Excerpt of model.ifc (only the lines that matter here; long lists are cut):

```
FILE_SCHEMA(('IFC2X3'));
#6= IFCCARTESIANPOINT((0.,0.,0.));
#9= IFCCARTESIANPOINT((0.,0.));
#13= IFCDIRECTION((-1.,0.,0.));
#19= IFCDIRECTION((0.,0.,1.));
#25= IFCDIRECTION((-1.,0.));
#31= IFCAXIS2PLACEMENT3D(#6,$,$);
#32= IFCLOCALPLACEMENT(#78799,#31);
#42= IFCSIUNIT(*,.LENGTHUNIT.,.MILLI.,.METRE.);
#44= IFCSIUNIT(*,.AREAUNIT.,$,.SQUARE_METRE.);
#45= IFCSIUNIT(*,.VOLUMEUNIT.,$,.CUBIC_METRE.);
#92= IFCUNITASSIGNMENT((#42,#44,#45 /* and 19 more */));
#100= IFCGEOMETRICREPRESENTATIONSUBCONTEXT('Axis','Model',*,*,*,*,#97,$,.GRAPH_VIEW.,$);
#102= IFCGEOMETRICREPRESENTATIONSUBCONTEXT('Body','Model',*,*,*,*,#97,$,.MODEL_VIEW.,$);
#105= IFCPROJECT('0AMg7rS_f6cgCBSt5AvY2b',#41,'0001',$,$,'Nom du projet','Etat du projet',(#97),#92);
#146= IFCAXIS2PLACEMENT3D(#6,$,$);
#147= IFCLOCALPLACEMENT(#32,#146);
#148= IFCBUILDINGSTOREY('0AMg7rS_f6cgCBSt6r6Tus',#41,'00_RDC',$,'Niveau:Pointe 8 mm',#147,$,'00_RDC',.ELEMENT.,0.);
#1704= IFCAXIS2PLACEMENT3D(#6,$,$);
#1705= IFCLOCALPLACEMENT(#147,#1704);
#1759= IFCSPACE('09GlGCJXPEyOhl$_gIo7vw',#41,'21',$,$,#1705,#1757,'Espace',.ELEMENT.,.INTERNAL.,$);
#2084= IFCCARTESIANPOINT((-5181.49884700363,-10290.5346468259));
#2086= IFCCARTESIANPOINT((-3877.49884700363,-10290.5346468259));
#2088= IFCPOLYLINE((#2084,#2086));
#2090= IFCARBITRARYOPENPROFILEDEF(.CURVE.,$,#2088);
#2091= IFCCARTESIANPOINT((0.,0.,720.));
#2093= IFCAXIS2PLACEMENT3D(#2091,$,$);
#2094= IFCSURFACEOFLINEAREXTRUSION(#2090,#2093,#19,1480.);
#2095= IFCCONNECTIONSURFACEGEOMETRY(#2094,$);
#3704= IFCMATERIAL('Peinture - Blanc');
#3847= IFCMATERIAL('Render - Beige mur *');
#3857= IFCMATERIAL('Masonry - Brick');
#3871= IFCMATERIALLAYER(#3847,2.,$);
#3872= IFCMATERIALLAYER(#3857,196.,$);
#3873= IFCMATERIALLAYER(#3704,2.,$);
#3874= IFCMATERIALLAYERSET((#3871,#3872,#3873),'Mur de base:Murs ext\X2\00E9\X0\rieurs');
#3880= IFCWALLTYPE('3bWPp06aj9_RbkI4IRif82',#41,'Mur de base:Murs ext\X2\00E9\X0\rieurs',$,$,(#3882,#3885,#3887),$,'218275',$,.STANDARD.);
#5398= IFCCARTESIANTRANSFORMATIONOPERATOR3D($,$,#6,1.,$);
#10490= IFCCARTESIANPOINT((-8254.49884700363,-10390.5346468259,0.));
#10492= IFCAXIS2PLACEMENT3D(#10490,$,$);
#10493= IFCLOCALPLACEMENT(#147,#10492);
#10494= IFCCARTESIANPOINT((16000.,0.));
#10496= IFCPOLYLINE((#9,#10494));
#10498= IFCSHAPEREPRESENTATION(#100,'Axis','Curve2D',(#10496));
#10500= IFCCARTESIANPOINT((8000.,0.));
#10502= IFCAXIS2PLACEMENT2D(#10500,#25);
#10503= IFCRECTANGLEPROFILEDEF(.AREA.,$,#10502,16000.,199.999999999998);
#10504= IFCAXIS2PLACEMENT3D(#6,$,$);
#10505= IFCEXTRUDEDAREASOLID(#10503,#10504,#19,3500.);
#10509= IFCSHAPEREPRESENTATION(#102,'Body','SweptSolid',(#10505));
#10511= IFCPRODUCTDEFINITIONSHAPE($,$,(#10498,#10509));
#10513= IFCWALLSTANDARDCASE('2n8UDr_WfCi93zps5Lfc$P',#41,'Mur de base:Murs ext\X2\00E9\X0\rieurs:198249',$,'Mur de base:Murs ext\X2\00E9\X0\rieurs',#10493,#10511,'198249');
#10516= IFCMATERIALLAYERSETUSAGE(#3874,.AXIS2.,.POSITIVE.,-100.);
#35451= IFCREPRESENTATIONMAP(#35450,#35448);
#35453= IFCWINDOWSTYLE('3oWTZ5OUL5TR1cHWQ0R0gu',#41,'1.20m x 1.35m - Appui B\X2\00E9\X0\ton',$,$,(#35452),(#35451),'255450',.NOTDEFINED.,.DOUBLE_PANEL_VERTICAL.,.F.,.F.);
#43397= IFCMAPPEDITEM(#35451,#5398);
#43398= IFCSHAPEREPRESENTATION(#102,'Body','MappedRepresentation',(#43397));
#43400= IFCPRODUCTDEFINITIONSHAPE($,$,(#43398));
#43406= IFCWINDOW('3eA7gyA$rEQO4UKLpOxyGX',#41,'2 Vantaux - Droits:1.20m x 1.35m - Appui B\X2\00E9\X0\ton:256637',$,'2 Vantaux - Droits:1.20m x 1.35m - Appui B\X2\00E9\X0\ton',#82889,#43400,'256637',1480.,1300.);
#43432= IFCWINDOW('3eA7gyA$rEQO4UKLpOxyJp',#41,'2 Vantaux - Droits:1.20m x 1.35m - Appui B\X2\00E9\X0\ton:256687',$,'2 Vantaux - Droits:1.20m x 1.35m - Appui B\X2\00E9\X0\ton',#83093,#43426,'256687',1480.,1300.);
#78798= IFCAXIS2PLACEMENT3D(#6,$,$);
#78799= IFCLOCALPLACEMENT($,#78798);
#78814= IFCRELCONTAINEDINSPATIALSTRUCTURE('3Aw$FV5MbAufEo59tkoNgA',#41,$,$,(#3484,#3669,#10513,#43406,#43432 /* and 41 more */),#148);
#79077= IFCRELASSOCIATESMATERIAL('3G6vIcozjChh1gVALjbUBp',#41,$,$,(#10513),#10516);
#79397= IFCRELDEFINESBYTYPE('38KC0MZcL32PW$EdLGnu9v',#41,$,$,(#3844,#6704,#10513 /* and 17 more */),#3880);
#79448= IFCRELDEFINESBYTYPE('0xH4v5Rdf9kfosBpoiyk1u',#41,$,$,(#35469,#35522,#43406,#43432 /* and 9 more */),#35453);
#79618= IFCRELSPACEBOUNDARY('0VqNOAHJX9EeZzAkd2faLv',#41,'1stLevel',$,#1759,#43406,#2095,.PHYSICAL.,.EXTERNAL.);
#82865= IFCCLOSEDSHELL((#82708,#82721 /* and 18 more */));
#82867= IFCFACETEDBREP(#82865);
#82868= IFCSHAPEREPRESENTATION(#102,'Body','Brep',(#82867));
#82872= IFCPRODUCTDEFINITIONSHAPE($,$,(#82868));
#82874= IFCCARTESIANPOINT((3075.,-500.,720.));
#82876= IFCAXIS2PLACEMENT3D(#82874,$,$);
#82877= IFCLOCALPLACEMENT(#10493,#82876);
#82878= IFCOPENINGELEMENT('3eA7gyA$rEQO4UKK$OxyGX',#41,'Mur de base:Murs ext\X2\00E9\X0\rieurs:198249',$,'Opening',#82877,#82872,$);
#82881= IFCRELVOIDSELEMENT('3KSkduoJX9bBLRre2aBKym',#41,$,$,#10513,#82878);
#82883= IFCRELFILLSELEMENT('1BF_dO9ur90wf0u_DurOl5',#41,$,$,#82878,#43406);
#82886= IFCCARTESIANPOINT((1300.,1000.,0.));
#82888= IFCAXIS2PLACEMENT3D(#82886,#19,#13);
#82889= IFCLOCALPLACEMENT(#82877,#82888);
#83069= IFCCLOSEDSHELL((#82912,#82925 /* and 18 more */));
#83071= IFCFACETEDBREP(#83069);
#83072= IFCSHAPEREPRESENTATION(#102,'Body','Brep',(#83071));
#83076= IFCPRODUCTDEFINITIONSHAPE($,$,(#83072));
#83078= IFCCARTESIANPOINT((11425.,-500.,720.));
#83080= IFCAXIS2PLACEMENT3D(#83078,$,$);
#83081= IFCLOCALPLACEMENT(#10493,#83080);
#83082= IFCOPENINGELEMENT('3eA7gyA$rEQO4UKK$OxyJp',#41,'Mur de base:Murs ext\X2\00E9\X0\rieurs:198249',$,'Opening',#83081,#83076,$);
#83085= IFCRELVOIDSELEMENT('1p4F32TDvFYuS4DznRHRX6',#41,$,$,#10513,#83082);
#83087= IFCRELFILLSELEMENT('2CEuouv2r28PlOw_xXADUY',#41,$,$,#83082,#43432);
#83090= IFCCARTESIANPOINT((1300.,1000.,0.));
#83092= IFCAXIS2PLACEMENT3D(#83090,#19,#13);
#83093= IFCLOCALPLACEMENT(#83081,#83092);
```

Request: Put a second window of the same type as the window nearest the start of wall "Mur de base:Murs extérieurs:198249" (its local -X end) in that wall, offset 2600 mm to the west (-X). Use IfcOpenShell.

```python
import numpy as np
import ifcopenshell
import ifcopenshell.api.feature
import ifcopenshell.api.geometry
import ifcopenshell.api.root
import ifcopenshell.geom
import ifcopenshell.util.element
import ifcopenshell.util.placement
import ifcopenshell.util.shape
import ifcopenshell.util.unit

model = ifcopenshell.open("model.ifc")
unit_scale = ifcopenshell.util.unit.calculate_unit_scale(model)
settings = ifcopenshell.geom.settings()


def volume(element):
    """Net volume in cubic metres, openings subtracted."""
    shape = ifcopenshell.geom.create_shape(settings, element)
    return ifcopenshell.util.shape.get_volume(shape.geometry)


def reuse_history(source, copy):
    """copy_class also copies each property set's owner history, people and application; keep the originals."""
    for rel in copy.IsDefinedBy:
        if rel.is_a("IfcRelDefinesByProperties") and (history := rel.RelatingPropertyDefinition.OwnerHistory):
            rel.RelatingPropertyDefinition.OwnerHistory = source.OwnerHistory
            ifcopenshell.util.element.remove_deep2(model, history)


window = model.by_guid("3eA7gyA$rEQO4UKLpOxyGX")
opening = window.FillsVoids[0].RelatingOpeningElement
wall = opening.VoidsElements[0].RelatingBuildingElement
before = volume(wall)
shift = ifcopenshell.util.placement.get_local_placement(wall.ObjectPlacement)[:3, 0] * -2.6 / unit_scale

# copy_class copies the void relationship, type, container and properties, but no geometry.
new_opening = ifcopenshell.api.root.copy_class(model, product=opening)
new_opening.Representation = ifcopenshell.util.element.copy_deep(
    model, opening.Representation, exclude=["IfcGeometricRepresentationContext", "IfcRepresentationMap"]
)
new_opening.Name = "Mur de base:Murs extérieurs"
new_window = ifcopenshell.api.root.copy_class(model, product=window)
new_window.Representation = ifcopenshell.util.element.copy_deep(
    model, window.Representation, exclude=["IfcGeometricRepresentationContext", "IfcRepresentationMap"]
)
new_window.Name = "2 Vantaux - Droits:1.20m x 1.35m - Appui Béton"
new_window.Tag = None
reuse_history(window, new_window)
fills = ifcopenshell.api.feature.add_filling(model, opening=new_opening, element=new_window)
fills.OwnerHistory = new_window.OwnerHistory  # required in IFC2X3

for old, new in ((opening, new_opening), (window, new_window)):
    matrix = ifcopenshell.util.placement.get_local_placement(old.ObjectPlacement)
    matrix[:3, 3] += shift
    ifcopenshell.api.geometry.edit_object_placement(model, product=new, matrix=matrix, is_si=False)

# The copied space boundaries still share their surfaces with the original.
for rel in new_window.ProvidesBoundaries:
    if rel.ConnectionGeometry:
        rel.ConnectionGeometry = ifcopenshell.util.element.copy_deep(model, rel.ConnectionGeometry)

# Space boundary surfaces are stored in each space's coordinates; move them too.
for rel in new_window.ProvidesBoundaries:
    if not rel.ConnectionGeometry:
        continue
    surface = rel.ConnectionGeometry.SurfaceOnRelatingElement
    space_matrix = ifcopenshell.util.placement.get_local_placement(rel.RelatingSpace.ObjectPlacement)
    point = np.array(surface.Position.Location.Coordinates) + space_matrix[:3, :3].T @ shift
    surface.Position = model.createIfcAxis2Placement3D(
        model.createIfcCartesianPoint(point.tolist()), surface.Position.Axis, surface.Position.RefDirection
    )

after = volume(wall)

print(f"wall volume {before:.3f} -> {after:.3f} m3")

model.write("model_updated.ifc")
```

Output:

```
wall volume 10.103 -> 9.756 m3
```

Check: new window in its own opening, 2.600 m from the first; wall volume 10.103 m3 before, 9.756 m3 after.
